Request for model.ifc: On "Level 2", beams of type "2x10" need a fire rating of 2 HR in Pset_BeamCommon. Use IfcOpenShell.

First a look at what the model holds.

```python
import ifcopenshell
import ifcopenshell.util.element

model = ifcopenshell.open("model.ifc")
print(model.schema)
storey = next(s for s in model.by_type("IfcBuildingStorey") if s.Name == "Level 2")
beams = [e for e in ifcopenshell.util.element.get_decomposition(storey) if e.is_a("IfcBeam")]
seen = {}
for e in beams:
    element_type = ifcopenshell.util.element.get_type(e)
    key = (element_type.Name if element_type != e and element_type else None, ifcopenshell.util.element.get_pset(e, "Pset_BeamCommon", "FireRating"))
    seen[key] = seen.get(key, 0) + 1
for (name, value), count in sorted(seen.items(), key=str):
    print(count, "x", name, "|", value)
```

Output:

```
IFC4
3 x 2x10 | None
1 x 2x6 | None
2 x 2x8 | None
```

```python
import ifcopenshell
import ifcopenshell.api.pset
import ifcopenshell.util.element

model = ifcopenshell.open("model.ifc")

storey = next(s for s in model.by_type("IfcBuildingStorey") if s.Name == "Level 2")
beams = [e for e in ifcopenshell.util.element.get_decomposition(storey) if e.is_a("IfcBeam")]

count = 0
for e in beams:
    element_type = ifcopenshell.util.element.get_type(e)
    if element_type in (None, e) or element_type.Name != "2x10":
        continue
    # add_pset returns the element's existing set when there is one.
    pset = ifcopenshell.api.pset.add_pset(model, product=e, name="Pset_BeamCommon")
    ifcopenshell.api.pset.edit_pset(model, pset=pset, properties={"FireRating": "2 HR"})
    count += 1

print(count, "beams updated")

model.write("model_v2.ifc")
```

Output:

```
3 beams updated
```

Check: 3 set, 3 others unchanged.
